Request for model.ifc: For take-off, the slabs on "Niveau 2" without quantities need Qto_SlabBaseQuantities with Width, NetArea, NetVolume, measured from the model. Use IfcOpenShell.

First a look at what the model holds.

```python
import ifcopenshell
import ifcopenshell.util.element
import ifcopenshell.util.unit

model = ifcopenshell.open("model.ifc")
print(model.schema)
for unit_type in ("LENGTHUNIT", "AREAUNIT", "VOLUMEUNIT"):
    print(unit_type, ifcopenshell.util.unit.calculate_unit_scale(model, unit_type))
storey = next(s for s in model.by_type("IfcBuildingStorey") if s.Name == "Niveau 2")
slabs = [e for e in ifcopenshell.util.element.get_decomposition(storey) if e.is_a("IfcSlab")]
for e in sorted(slabs, key=lambda e: e.id()):
    print(e.id(), e.is_a(), e.Name, list(ifcopenshell.util.element.get_psets(e, qtos_only=True)), sep=" | ")
```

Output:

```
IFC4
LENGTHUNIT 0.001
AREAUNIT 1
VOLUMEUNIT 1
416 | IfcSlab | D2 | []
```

```python
import ifcopenshell
import ifcopenshell.api.pset
import ifcopenshell.geom
import ifcopenshell.util.element
import ifcopenshell.util.shape
import ifcopenshell.util.unit

model = ifcopenshell.open("model.ifc")
unit_scale = ifcopenshell.util.unit.calculate_unit_scale(model)
area_scale = ifcopenshell.util.unit.calculate_unit_scale(model, "AREAUNIT")
volume_scale = ifcopenshell.util.unit.calculate_unit_scale(model, "VOLUMEUNIT")
settings = ifcopenshell.geom.settings()

storey = next(s for s in model.by_type("IfcBuildingStorey") if s.Name == "Niveau 2")
slabs = [e for e in ifcopenshell.util.element.get_decomposition(storey) if e.is_a("IfcSlab")]

for e in sorted(slabs, key=lambda e: e.id()):
    if ifcopenshell.util.element.get_psets(e, qtos_only=True, should_inherit=False):
        continue
    # Geometry comes back in metres, in the element's own axes.
    shape = ifcopenshell.geom.create_shape(settings, e)
    values = {
        "Width": ifcopenshell.util.shape.get_z(shape.geometry) / unit_scale,
        "NetArea": ifcopenshell.util.shape.get_footprint_area(shape.geometry) / area_scale,
        "NetVolume": ifcopenshell.util.shape.get_volume(shape.geometry) / volume_scale,
    }
    qto = ifcopenshell.api.pset.add_qto(model, product=e, name="Qto_SlabBaseQuantities")
    ifcopenshell.api.pset.edit_qto(model, qto=qto, properties=values)
    print(e.id(), {k: round(v, 3) for k, v in values.items()})

model.write("model_updated.ifc")
```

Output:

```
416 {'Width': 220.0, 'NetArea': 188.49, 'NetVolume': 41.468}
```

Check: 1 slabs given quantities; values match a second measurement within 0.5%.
